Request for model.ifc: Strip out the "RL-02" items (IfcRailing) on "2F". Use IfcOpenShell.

First a look at what the model holds.

```python
import ifcopenshell
import ifcopenshell.util.element

model = ifcopenshell.open("model.ifc")
print(model.schema)
storey = next(s for s in model.by_type("IfcBuildingStorey") if s.Name == "2F")
railings = [e for e in ifcopenshell.util.element.get_decomposition(storey) if e.is_a("IfcRailing")]
seen = {}
for e in railings:
    element_type = ifcopenshell.util.element.get_type(e)
    name = element_type.Name if element_type not in (None, e) else None
    seen[name] = seen.get(name, 0) + 1
for name, count in sorted(seen.items(), key=str):
    print(count, "x", name)
```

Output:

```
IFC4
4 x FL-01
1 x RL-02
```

```python
import ifcopenshell
import ifcopenshell.api.root
import ifcopenshell.util.element

model = ifcopenshell.open("model.ifc")

storey = next(s for s in model.by_type("IfcBuildingStorey") if s.Name == "2F")
railings = [e for e in ifcopenshell.util.element.get_decomposition(storey) if e.is_a("IfcRailing")]
targets = [e for e in railings if (t := ifcopenshell.util.element.get_type(e)) not in (None, e) and t.Name == "RL-02"]

for e in targets:
    ifcopenshell.api.root.remove_product(model, product=e)
print(len(targets), "removed")

model.write("model-out.ifc")
```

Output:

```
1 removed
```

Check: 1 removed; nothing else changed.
